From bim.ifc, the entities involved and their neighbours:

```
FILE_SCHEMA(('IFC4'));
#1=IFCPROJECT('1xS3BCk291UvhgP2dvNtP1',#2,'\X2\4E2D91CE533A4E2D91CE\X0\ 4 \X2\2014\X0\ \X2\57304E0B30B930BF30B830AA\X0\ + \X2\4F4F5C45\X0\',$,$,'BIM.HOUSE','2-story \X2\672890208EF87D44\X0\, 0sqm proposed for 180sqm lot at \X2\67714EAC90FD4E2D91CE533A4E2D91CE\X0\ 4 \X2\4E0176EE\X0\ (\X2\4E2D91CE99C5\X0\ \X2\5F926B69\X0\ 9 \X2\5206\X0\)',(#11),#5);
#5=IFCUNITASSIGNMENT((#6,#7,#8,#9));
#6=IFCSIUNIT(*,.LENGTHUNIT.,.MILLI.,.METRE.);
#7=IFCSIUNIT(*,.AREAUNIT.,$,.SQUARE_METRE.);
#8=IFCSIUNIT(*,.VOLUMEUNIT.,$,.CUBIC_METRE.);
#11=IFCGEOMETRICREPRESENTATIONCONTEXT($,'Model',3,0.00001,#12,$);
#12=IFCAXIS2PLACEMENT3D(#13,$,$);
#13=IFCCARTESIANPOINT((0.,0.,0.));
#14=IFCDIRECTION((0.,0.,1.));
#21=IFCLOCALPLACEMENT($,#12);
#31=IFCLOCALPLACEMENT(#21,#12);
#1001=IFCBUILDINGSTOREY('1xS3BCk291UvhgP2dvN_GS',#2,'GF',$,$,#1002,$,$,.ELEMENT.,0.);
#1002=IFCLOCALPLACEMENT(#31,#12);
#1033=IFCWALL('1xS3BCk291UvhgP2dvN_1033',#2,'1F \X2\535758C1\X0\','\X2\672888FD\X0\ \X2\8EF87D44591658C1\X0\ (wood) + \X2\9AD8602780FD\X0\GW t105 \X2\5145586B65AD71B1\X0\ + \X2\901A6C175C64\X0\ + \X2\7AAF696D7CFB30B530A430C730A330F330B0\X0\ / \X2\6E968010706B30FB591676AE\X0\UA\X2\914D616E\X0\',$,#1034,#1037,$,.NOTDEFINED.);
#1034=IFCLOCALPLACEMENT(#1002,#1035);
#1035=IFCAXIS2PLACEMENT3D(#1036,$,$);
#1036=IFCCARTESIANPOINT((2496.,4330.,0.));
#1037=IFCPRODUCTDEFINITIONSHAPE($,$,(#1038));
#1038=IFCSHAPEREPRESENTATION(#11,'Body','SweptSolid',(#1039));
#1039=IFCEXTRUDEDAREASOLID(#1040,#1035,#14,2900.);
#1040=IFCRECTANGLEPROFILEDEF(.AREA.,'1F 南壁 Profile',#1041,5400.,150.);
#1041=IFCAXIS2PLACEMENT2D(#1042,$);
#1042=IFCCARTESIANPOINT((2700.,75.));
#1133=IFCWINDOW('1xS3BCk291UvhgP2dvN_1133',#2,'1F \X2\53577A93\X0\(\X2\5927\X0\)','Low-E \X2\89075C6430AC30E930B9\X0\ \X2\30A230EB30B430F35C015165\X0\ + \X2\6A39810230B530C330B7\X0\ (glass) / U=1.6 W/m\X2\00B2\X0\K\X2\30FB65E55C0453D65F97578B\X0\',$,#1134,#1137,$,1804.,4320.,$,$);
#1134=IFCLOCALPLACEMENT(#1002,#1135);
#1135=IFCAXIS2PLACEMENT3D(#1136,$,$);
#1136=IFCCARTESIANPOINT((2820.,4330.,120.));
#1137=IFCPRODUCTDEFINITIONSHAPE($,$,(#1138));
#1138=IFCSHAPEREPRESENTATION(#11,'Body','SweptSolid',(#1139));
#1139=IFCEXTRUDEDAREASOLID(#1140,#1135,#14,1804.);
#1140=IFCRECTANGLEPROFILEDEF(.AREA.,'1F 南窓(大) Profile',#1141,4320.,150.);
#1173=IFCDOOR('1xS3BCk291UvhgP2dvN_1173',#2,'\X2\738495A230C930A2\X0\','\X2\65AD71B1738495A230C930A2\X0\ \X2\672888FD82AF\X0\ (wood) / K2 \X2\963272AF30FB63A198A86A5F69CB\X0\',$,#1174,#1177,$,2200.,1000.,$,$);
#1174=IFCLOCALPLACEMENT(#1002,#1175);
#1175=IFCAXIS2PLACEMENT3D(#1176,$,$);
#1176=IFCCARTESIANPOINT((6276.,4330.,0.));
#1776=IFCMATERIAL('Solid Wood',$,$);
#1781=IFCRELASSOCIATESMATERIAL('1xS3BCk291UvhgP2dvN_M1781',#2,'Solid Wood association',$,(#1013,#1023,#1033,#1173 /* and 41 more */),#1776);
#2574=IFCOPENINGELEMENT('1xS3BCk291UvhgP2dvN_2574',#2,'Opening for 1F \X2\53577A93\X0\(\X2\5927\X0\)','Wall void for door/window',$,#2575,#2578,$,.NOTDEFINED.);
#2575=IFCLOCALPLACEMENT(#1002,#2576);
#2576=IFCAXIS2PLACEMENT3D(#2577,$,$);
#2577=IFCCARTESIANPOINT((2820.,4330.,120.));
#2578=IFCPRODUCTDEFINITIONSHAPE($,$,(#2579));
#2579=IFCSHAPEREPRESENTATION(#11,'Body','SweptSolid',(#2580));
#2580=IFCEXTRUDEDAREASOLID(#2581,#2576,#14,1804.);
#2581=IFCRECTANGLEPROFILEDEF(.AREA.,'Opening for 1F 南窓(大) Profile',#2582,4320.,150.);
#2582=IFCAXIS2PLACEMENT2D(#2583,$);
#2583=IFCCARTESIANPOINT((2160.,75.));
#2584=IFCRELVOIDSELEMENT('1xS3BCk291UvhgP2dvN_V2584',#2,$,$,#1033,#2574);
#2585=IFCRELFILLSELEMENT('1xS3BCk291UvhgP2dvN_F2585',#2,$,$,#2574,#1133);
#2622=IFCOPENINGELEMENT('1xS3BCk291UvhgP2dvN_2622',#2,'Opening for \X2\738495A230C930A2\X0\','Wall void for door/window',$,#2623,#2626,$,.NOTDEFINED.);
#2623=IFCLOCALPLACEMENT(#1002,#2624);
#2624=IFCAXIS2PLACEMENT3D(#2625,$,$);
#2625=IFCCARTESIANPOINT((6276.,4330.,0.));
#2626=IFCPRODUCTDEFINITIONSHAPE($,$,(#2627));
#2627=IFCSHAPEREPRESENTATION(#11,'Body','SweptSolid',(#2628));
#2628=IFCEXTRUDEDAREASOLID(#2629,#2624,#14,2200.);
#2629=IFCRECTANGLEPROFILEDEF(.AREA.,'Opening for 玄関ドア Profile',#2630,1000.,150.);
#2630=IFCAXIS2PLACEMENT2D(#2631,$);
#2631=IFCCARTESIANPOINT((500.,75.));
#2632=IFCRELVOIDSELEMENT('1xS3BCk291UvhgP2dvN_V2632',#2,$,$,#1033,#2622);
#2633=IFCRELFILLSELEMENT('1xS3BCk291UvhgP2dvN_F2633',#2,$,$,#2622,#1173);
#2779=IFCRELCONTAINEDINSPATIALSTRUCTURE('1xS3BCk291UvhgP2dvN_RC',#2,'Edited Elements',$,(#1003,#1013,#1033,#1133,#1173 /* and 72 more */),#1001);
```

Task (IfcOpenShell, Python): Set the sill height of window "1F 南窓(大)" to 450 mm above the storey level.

```python
import numpy as np
import ifcopenshell
import ifcopenshell.api.geometry
import ifcopenshell.geom
import ifcopenshell.util.element
import ifcopenshell.util.placement
import ifcopenshell.util.shape
import ifcopenshell.util.unit

model = ifcopenshell.open("bim.ifc")
unit_scale = ifcopenshell.util.unit.calculate_unit_scale(model)

window = model.by_id(1133)
opening = window.FillsVoids[0].RelatingOpeningElement
storey = ifcopenshell.util.element.get_container(window, ifc_class="IfcBuildingStorey")
level = ifcopenshell.util.placement.get_local_placement(storey.ObjectPlacement)[2, 3]

# The opening's origin need not be at the sill, so measure its lowest point.
shape = ifcopenshell.geom.create_shape(ifcopenshell.geom.settings(), opening)
bottom = ifcopenshell.util.shape.get_shape_bottom_elevation(shape, shape.geometry) / unit_scale
dz = level + 0.45 / unit_scale - bottom

shift = np.array([0.0, 0.0, dz])
# The window is not placed relative to its opening, so move both.
for product in (opening, window):
    matrix = ifcopenshell.util.placement.get_local_placement(product.ObjectPlacement)
    matrix[:3, 3] += shift
    ifcopenshell.api.geometry.edit_object_placement(model, product=product, matrix=matrix, is_si=False)

print(f"moved by {dz * unit_scale:+.3f} m")

model.write("bim_v2.ifc")
```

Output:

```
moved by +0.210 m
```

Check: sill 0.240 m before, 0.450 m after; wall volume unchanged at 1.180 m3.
